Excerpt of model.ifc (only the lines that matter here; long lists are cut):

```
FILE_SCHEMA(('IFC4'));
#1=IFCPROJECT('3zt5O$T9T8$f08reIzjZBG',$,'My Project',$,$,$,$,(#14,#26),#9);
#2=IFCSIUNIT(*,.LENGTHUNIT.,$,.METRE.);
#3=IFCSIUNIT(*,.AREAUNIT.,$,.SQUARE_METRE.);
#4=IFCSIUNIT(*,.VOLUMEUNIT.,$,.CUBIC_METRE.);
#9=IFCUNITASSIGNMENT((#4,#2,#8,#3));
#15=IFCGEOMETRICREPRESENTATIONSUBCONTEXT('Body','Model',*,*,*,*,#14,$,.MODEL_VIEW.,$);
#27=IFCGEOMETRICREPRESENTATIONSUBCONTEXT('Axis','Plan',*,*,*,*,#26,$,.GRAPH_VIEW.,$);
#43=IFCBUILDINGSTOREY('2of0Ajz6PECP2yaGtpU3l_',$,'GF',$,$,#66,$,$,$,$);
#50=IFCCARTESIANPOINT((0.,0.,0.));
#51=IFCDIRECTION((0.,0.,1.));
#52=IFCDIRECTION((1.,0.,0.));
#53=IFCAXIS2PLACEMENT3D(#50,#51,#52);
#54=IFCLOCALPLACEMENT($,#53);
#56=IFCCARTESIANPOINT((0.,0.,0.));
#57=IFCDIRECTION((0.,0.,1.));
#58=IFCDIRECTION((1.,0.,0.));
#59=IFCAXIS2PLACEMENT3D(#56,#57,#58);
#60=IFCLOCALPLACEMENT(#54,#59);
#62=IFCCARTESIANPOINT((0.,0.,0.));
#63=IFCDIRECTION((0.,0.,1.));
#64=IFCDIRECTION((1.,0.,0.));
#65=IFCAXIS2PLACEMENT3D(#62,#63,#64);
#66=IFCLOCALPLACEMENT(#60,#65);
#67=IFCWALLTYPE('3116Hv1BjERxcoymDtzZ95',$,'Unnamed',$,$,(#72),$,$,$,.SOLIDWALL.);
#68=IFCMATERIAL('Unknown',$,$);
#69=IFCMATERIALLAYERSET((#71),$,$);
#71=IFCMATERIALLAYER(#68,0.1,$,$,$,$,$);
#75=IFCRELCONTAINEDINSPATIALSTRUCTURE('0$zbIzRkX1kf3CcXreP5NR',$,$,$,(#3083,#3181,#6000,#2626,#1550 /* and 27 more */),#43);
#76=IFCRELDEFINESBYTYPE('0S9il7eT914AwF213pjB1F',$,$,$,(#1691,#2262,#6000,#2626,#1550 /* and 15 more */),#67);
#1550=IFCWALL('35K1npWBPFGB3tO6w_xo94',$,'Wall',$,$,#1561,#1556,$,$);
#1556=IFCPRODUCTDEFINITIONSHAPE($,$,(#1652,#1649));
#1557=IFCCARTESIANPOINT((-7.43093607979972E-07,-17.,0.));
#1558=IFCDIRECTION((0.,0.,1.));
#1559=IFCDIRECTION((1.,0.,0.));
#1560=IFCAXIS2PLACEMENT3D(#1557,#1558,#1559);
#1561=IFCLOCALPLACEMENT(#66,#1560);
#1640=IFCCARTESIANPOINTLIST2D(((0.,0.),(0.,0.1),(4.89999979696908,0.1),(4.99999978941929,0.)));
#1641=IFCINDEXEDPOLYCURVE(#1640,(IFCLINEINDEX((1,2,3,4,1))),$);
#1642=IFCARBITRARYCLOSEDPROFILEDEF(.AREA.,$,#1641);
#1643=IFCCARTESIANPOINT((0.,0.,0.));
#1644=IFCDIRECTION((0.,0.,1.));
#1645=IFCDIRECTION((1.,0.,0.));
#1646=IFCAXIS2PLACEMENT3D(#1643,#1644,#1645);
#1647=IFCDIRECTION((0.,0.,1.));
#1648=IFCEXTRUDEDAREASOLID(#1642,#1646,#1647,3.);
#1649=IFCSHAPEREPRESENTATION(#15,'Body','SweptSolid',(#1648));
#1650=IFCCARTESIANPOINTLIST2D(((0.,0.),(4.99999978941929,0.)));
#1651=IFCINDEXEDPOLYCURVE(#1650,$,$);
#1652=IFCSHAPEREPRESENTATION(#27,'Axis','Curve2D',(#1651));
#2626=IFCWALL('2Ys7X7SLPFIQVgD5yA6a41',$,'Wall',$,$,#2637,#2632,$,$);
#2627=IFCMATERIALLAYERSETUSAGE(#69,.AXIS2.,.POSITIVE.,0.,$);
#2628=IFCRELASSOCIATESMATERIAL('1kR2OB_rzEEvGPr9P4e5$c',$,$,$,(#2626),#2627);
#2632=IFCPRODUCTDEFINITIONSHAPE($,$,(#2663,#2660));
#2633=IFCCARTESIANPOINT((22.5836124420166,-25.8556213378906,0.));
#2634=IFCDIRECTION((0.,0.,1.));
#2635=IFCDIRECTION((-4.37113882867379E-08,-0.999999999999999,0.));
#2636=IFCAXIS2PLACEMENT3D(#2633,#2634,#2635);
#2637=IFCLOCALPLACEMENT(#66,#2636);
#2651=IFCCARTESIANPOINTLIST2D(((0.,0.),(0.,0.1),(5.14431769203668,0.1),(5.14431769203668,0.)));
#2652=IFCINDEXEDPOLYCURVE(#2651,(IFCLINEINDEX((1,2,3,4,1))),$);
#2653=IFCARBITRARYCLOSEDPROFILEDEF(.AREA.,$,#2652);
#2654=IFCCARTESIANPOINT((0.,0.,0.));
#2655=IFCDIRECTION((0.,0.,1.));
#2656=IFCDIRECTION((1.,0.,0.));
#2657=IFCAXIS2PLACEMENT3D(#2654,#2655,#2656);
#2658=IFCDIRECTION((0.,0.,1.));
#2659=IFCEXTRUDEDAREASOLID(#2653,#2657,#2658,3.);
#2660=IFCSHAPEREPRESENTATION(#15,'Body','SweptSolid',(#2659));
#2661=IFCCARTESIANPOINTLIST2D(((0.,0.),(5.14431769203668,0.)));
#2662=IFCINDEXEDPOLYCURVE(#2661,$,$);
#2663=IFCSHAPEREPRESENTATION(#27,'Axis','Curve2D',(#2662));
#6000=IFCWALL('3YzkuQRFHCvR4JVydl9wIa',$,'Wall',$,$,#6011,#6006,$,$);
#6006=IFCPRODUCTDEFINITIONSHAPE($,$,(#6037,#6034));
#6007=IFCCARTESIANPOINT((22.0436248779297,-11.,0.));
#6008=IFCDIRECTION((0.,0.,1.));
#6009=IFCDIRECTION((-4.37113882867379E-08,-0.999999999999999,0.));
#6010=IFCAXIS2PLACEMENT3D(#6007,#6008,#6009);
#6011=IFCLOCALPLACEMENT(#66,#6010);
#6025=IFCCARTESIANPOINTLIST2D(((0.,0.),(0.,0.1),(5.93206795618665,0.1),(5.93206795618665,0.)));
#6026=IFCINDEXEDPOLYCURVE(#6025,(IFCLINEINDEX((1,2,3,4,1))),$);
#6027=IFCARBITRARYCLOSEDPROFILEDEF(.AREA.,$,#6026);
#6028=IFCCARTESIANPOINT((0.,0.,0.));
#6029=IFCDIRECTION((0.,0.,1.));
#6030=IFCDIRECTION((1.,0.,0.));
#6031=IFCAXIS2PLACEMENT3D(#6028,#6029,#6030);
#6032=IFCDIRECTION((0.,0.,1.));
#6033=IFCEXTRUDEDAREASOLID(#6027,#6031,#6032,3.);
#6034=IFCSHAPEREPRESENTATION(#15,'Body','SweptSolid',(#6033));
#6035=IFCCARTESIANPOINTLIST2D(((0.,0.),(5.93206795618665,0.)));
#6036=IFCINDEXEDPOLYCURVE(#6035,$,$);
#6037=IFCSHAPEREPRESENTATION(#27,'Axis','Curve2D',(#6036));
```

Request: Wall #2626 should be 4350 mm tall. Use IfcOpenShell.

```python
import ifcopenshell
import ifcopenshell.geom
import ifcopenshell.util.representation
import ifcopenshell.util.shape
import ifcopenshell.util.unit

model = ifcopenshell.open("model.ifc")
unit_scale = ifcopenshell.util.unit.calculate_unit_scale(model)
settings = ifcopenshell.geom.settings()


def volume(element):
    """Net volume in cubic metres, openings subtracted."""
    shape = ifcopenshell.geom.create_shape(settings, element)
    return ifcopenshell.util.shape.get_volume(shape.geometry)


wall = model.by_guid("2Ys7X7SLPFIQVgD5yA6a41")
before = volume(wall)

body = ifcopenshell.util.representation.get_representation(wall, "Model", "Body")
solid = body.Items[0]
old_height = solid.Depth
solid.Depth = 4.35 / unit_scale
after = volume(wall)

print(f"height {old_height:g} -> {solid.Depth:g}, volume {before:.3f} -> {after:.3f} m3")

model.write("model_edited.ifc")
```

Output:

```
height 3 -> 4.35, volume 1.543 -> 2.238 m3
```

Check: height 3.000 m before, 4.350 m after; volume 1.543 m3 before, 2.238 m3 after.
